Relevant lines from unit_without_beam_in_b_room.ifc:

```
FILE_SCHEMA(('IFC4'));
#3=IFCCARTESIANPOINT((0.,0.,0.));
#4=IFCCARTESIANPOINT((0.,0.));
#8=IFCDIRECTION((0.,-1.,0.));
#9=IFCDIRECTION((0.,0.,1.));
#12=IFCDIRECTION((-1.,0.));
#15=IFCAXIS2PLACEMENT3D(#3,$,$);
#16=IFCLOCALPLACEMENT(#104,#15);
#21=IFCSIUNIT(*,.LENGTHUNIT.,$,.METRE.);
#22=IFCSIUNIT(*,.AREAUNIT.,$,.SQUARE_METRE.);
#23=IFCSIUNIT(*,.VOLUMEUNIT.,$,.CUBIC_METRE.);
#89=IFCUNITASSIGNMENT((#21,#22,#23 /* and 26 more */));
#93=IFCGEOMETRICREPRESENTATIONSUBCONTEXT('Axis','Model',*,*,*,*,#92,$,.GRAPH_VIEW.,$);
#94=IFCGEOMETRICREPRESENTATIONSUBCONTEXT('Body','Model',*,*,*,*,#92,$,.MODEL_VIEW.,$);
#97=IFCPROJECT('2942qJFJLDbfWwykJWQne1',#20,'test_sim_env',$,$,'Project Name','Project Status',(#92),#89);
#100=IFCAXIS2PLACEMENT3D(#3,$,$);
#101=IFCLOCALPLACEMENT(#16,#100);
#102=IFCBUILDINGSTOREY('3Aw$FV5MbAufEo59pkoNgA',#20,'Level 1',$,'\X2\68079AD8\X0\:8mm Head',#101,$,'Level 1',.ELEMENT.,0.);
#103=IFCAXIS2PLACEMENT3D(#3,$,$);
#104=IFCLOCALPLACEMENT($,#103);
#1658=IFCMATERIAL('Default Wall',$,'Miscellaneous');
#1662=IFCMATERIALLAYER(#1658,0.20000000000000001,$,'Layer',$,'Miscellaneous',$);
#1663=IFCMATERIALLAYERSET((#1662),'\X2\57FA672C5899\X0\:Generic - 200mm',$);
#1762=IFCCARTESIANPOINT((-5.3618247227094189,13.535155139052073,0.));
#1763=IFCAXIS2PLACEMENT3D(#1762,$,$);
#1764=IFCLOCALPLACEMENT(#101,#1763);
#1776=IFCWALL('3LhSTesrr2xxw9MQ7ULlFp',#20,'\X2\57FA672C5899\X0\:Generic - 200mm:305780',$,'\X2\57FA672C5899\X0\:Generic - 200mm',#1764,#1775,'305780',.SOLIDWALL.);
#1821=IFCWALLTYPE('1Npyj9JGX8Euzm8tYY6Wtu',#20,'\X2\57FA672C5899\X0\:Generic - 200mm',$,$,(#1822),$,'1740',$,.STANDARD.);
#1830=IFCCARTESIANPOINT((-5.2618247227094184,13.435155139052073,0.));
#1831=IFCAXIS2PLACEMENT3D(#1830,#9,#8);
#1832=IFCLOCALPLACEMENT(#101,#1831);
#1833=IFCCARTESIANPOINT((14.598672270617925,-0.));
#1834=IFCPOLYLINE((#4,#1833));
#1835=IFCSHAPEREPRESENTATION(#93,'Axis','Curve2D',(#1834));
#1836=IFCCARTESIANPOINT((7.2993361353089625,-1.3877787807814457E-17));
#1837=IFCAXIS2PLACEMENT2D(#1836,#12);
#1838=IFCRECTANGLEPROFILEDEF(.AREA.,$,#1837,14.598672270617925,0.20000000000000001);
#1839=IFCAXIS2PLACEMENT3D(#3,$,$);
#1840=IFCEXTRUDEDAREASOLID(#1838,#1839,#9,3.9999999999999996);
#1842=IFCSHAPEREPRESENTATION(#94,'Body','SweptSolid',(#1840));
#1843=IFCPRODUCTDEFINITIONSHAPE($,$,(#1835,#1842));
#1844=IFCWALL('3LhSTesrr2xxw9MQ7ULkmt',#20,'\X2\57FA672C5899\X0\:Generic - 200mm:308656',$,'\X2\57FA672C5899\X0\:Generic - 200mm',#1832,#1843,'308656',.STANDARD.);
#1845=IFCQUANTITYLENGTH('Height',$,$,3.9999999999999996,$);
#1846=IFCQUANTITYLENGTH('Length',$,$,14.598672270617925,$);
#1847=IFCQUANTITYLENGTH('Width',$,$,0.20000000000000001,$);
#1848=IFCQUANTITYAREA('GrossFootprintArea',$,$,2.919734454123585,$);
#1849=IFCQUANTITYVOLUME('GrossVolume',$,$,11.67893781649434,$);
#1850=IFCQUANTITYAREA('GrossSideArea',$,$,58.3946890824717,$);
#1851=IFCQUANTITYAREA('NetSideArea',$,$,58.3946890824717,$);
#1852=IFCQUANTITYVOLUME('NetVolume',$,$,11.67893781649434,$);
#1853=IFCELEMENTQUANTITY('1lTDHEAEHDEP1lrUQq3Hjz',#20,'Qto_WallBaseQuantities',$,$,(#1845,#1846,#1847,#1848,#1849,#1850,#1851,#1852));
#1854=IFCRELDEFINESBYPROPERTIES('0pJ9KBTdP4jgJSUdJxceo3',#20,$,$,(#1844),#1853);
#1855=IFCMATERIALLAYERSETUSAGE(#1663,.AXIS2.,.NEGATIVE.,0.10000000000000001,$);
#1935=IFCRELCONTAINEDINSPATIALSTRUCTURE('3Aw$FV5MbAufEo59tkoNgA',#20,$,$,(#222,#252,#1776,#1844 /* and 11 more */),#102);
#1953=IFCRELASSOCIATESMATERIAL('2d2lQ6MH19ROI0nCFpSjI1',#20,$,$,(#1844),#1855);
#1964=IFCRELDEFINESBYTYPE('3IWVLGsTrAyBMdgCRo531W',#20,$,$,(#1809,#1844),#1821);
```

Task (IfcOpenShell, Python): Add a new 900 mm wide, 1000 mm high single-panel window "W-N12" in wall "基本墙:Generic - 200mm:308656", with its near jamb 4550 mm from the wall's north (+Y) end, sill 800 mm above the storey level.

```python
import numpy as np
import ifcopenshell
import ifcopenshell.api.feature
import ifcopenshell.api.geometry
import ifcopenshell.api.pset
import ifcopenshell.api.root
import ifcopenshell.api.spatial
import ifcopenshell.geom
import ifcopenshell.util.element
import ifcopenshell.util.placement
import ifcopenshell.util.representation
import ifcopenshell.util.shape
import ifcopenshell.util.unit

model = ifcopenshell.open("unit_without_beam_in_b_room.ifc")
unit_scale = ifcopenshell.util.unit.calculate_unit_scale(model)
area_scale = ifcopenshell.util.unit.calculate_unit_scale(model, "AREAUNIT")
volume_scale = ifcopenshell.util.unit.calculate_unit_scale(model, "VOLUMEUNIT")
settings = ifcopenshell.geom.settings()


def volume(element):
    """Net volume in cubic metres, openings subtracted."""
    shape = ifcopenshell.geom.create_shape(settings, element)
    return ifcopenshell.util.shape.get_volume(shape.geometry)


wall = model.by_guid("3LhSTesrr2xxw9MQ7ULkmt")
storey = ifcopenshell.util.element.get_container(wall, ifc_class="IfcBuildingStorey")
context = ifcopenshell.util.representation.get_context(model, "Model", "Body", "MODEL_VIEW")
before = volume(wall)

width, height, from_end, sill = 0.9, 1, 4.55, 0.8  # metres

# The wall runs along its own X axis, and the end named is its -X end.
wall_shape = ifcopenshell.geom.create_shape(settings, wall)
x, y, z = ifcopenshell.util.shape.get_vertices(wall_shape.geometry).T
start = x.min() + from_end
face, thickness = float(y.min()), float(y.max() - y.min())
wall_matrix = ifcopenshell.util.placement.get_local_placement(wall.ObjectPlacement)
level = ifcopenshell.util.placement.get_local_placement(storey.ObjectPlacement)[2, 3]


def in_wall(x, y):
    """Placement at x, y metres in the wall's axes, at sill height."""
    matrix = wall_matrix.copy()
    matrix[:, 3] = wall_matrix @ np.array([x / unit_scale, y / unit_scale, 0.0, 1.0])
    matrix[2, 3] = level + sill / unit_scale
    return matrix


# Opening: a box that overshoots both wall faces by 50 mm.
opening = ifcopenshell.api.root.create_entity(model, ifc_class="IfcOpeningElement", predefined_type="OPENING")
box = ifcopenshell.api.geometry.add_wall_representation(
    model, context=context, length=width, height=height, thickness=thickness + 0.1
)
ifcopenshell.api.geometry.assign_representation(model, product=opening, representation=box)
ifcopenshell.api.geometry.edit_object_placement(model, product=opening, matrix=in_wall(start, face - 0.05), is_si=False)
ifcopenshell.api.feature.add_feature(model, feature=opening, element=wall)

window = ifcopenshell.api.root.create_entity(model, ifc_class="IfcWindow", name="W-N12", predefined_type="WINDOW")
window.OverallWidth, window.OverallHeight = width / unit_scale, height / unit_scale
window.PartitioningType = "SINGLE_PANEL"
body = ifcopenshell.api.geometry.add_window_representation(
    model,
    context=context,
    overall_width=window.OverallWidth,
    overall_height=window.OverallHeight,
    partition_type="SINGLE_PANEL",
)
ifcopenshell.api.geometry.assign_representation(model, product=window, representation=body)
ifcopenshell.api.spatial.assign_container(model, products=[window], relating_structure=storey)
ifcopenshell.api.feature.add_filling(model, opening=opening, element=window)

# Centre the window in the wall's thickness.
ifcopenshell.api.geometry.edit_object_placement(model, product=window, matrix=in_wall(start, face), is_si=False)
window_shape = ifcopenshell.geom.create_shape(settings, window)
depth = ifcopenshell.util.shape.get_vertices(window_shape.geometry)[:, 1]
offset = face + thickness / 2 - (depth.min() + depth.max()) / 2
ifcopenshell.api.geometry.edit_object_placement(model, product=window, matrix=in_wall(start, offset), is_si=False)

after = volume(wall)

# Update the wall's stored quantities.
qto = model.by_id(ifcopenshell.util.element.get_pset(wall, "Qto_WallBaseQuantities", should_inherit=False)["id"])
ifcopenshell.api.pset.edit_qto(model, qto=qto, properties={
    "NetSideArea": after / thickness / area_scale,
    "NetVolume": after / volume_scale,
})

print(f"wall volume {before:.3f} -> {after:.3f} m3")

model.write("unit_without_beam_in_b_room_updated.ifc")
```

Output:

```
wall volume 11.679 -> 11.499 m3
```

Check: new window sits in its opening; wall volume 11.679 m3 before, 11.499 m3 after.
